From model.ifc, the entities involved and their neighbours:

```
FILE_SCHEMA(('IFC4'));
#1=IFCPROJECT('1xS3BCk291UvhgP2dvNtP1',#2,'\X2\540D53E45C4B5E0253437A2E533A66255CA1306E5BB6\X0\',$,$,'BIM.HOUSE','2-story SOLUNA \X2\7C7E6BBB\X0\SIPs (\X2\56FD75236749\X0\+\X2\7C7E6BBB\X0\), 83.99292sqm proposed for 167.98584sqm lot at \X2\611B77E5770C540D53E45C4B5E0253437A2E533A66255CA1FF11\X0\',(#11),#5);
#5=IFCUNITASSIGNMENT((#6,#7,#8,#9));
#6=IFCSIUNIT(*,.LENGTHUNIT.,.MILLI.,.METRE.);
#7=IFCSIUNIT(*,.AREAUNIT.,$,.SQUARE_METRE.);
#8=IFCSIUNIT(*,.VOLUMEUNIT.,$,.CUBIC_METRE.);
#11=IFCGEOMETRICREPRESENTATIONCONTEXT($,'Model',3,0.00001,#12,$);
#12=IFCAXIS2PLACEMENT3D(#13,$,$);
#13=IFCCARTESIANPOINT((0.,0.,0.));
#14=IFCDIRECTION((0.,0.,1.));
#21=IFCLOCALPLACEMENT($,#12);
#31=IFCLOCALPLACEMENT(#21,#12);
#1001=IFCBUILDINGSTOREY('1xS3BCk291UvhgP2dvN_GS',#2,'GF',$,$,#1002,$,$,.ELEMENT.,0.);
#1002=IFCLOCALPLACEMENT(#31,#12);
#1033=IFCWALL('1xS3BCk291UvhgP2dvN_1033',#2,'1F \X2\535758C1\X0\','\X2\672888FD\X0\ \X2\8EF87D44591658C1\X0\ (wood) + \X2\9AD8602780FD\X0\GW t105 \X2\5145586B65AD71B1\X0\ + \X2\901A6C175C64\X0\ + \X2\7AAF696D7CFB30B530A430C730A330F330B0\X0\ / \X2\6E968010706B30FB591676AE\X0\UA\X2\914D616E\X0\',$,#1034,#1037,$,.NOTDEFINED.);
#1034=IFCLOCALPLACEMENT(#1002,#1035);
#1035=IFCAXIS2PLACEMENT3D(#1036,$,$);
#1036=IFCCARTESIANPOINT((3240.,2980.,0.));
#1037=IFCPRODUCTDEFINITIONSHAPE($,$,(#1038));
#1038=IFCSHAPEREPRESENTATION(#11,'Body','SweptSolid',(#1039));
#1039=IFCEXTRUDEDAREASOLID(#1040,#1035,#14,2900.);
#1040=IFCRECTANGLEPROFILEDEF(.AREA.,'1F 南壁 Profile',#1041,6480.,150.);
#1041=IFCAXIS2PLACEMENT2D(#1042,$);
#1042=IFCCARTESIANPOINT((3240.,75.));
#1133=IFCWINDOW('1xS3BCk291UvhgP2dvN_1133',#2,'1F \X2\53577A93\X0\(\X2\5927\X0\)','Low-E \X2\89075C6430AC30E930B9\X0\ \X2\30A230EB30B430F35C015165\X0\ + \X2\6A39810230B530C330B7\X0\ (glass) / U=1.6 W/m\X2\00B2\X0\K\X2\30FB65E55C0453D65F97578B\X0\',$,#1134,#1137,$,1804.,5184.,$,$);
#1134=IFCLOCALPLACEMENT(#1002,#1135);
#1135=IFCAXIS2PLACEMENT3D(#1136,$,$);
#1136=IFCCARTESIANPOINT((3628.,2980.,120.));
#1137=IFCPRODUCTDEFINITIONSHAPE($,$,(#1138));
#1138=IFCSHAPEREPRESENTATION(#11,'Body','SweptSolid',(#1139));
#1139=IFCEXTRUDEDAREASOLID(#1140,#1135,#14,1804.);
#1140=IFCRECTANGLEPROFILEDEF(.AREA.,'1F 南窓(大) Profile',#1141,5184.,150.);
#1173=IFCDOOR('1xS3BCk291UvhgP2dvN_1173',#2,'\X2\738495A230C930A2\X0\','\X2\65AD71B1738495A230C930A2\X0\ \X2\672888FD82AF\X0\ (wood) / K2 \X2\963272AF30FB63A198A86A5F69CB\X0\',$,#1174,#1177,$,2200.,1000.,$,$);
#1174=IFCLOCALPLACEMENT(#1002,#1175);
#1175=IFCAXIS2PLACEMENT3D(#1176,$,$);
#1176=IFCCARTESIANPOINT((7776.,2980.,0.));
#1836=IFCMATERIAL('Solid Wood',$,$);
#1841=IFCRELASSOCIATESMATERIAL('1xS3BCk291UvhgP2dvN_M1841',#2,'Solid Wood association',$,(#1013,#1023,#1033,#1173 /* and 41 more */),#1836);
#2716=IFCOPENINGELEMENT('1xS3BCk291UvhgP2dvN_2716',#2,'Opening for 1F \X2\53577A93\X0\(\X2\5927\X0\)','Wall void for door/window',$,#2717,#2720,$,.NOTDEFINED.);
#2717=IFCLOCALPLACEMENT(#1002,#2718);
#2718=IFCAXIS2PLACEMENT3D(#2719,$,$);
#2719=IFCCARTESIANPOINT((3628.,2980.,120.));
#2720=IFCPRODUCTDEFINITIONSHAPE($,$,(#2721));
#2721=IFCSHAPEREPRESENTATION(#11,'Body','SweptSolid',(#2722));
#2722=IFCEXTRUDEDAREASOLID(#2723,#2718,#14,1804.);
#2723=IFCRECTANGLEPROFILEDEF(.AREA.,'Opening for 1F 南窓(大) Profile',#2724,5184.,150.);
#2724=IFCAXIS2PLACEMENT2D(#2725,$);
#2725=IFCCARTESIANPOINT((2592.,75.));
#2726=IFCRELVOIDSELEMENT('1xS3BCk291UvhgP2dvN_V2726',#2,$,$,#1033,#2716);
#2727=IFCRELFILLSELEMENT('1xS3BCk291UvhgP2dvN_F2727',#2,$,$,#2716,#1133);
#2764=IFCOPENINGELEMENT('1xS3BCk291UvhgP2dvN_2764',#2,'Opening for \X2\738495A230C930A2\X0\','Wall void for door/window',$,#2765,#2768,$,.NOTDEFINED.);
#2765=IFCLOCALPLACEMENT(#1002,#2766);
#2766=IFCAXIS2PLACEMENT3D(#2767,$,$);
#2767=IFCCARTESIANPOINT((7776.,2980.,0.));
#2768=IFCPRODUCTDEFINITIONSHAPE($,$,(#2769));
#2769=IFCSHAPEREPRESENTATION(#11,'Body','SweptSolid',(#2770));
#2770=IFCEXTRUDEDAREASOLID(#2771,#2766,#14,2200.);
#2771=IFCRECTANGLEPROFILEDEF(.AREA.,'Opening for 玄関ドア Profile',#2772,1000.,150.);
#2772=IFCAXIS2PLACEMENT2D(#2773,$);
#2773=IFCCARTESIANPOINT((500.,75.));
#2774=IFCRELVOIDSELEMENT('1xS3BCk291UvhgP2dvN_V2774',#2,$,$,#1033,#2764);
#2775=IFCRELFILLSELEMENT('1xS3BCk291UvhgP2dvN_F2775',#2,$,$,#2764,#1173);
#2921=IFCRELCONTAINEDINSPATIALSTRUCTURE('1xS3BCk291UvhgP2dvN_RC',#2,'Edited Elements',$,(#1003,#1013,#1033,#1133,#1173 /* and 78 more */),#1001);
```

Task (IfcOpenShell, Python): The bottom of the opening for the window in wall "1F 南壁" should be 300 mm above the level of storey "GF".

```python
import numpy as np
import ifcopenshell
import ifcopenshell.api.geometry
import ifcopenshell.geom
import ifcopenshell.util.element
import ifcopenshell.util.placement
import ifcopenshell.util.shape
import ifcopenshell.util.unit

model = ifcopenshell.open("model.ifc")
unit_scale = ifcopenshell.util.unit.calculate_unit_scale(model)

window = model.by_guid("1xS3BCk291UvhgP2dvN_1133")
opening = window.FillsVoids[0].RelatingOpeningElement
storey = ifcopenshell.util.element.get_container(window, ifc_class="IfcBuildingStorey")
level = ifcopenshell.util.placement.get_local_placement(storey.ObjectPlacement)[2, 3]

# The opening's origin need not be at the sill, so measure its lowest point.
shape = ifcopenshell.geom.create_shape(ifcopenshell.geom.settings(), opening)
bottom = ifcopenshell.util.shape.get_shape_bottom_elevation(shape, shape.geometry) / unit_scale
dz = level + 0.3 / unit_scale - bottom

shift = np.array([0.0, 0.0, dz])
# The window is not placed relative to its opening, so move both.
for product in (opening, window):
    matrix = ifcopenshell.util.placement.get_local_placement(product.ObjectPlacement)
    matrix[:3, 3] += shift
    ifcopenshell.api.geometry.edit_object_placement(model, product=product, matrix=matrix, is_si=False)

print(f"moved by {dz * unit_scale:+.3f} m")

model.write("model_v2.ifc")
```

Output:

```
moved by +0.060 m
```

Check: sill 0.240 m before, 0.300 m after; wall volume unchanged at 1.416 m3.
